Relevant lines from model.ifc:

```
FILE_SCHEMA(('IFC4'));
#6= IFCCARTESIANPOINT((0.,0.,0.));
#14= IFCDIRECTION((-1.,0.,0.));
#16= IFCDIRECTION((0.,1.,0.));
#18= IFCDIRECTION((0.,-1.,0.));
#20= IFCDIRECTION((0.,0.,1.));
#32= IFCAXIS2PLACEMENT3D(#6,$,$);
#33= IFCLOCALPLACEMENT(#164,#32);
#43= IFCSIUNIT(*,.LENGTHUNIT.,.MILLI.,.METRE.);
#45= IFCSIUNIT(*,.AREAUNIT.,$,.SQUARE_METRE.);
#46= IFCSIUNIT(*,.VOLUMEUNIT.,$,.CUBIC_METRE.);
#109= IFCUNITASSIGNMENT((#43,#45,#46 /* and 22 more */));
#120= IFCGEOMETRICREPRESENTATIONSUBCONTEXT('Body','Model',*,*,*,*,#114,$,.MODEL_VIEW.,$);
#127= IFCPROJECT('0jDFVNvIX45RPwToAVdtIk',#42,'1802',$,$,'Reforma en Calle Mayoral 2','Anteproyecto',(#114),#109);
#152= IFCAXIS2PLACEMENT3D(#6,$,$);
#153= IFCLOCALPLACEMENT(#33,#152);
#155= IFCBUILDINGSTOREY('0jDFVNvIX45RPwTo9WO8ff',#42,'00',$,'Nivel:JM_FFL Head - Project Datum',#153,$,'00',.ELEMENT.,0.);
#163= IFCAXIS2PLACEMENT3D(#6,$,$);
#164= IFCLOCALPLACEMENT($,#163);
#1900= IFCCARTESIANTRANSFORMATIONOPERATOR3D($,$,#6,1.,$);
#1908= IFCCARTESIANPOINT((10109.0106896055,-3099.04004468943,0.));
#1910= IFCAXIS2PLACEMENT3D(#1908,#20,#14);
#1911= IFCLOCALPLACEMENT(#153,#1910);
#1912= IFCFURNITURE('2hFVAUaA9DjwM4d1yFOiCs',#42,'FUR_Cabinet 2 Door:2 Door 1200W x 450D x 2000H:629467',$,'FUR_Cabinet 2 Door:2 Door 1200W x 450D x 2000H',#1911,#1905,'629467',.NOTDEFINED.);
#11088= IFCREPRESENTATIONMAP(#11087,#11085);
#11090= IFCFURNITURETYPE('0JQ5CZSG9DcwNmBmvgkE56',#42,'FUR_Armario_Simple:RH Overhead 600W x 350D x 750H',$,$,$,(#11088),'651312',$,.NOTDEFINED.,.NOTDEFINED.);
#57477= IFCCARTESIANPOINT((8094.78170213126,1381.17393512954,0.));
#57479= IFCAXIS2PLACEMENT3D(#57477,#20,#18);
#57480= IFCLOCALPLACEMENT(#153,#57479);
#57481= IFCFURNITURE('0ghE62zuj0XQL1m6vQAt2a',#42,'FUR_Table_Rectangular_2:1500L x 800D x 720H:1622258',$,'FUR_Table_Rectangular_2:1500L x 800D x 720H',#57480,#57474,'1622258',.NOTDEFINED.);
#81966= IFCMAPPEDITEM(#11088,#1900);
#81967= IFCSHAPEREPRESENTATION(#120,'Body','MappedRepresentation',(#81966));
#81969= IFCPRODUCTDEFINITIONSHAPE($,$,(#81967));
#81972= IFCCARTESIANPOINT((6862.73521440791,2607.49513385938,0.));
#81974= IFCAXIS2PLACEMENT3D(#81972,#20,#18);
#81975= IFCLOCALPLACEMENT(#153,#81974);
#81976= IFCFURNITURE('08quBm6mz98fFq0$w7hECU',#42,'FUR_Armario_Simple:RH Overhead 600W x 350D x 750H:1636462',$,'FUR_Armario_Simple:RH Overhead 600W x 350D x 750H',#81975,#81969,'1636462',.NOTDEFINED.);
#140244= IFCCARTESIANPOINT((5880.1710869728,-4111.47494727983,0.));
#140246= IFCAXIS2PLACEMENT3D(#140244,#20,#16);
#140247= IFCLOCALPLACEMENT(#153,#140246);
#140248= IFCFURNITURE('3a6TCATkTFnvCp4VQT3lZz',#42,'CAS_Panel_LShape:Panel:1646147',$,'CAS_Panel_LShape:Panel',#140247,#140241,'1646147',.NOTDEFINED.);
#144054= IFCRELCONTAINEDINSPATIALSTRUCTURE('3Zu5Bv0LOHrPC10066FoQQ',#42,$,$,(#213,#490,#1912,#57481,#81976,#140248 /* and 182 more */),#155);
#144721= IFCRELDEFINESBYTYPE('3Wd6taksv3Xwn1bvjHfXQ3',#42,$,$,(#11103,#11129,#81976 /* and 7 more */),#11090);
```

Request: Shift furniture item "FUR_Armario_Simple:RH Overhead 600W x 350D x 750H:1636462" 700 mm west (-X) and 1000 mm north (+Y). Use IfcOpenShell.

```python
import ifcopenshell
import ifcopenshell.api.geometry
import ifcopenshell.util.placement

model = ifcopenshell.open("model.ifc")

item = model.by_id(81976)
matrix = ifcopenshell.util.placement.get_local_placement(item.ObjectPlacement)
matrix[0, 3] -= 700.0
matrix[1, 3] += 1000.0
ifcopenshell.api.geometry.edit_object_placement(model, product=item, matrix=matrix, is_si=False)

print(ifcopenshell.util.placement.get_local_placement(item.ObjectPlacement).round(3) + 0.0)

model.write("model_rev.ifc")
```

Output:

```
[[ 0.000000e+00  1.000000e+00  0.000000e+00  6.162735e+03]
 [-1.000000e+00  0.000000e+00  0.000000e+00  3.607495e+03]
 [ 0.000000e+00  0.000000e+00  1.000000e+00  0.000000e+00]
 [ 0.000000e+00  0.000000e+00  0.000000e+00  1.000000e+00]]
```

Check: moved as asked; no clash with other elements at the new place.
